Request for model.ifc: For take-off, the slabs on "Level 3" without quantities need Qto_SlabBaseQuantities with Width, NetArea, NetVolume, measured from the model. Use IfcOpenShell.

First a look at what the model holds.

```python
import ifcopenshell
import ifcopenshell.util.element
import ifcopenshell.util.unit

model = ifcopenshell.open("model.ifc")
print(model.schema)
for unit_type in ("LENGTHUNIT", "AREAUNIT", "VOLUMEUNIT"):
    print(unit_type, ifcopenshell.util.unit.calculate_unit_scale(model, unit_type))
storey = next(s for s in model.by_type("IfcBuildingStorey") if s.Name == "Level 3")
slabs = [e for e in ifcopenshell.util.element.get_decomposition(storey) if e.is_a("IfcSlab")]
for e in sorted(slabs, key=lambda e: e.id()):
    print(e.id(), e.is_a(), e.Name, list(ifcopenshell.util.element.get_psets(e, qtos_only=True)), sep=" | ")
```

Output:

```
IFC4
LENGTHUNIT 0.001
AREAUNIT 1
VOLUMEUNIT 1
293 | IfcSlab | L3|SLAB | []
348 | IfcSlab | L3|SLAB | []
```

```python
import ifcopenshell
import ifcopenshell.api.pset
import ifcopenshell.geom
import ifcopenshell.util.element
import ifcopenshell.util.shape
import ifcopenshell.util.unit

model = ifcopenshell.open("model.ifc")
unit_scale = ifcopenshell.util.unit.calculate_unit_scale(model)
area_scale = ifcopenshell.util.unit.calculate_unit_scale(model, "AREAUNIT")
volume_scale = ifcopenshell.util.unit.calculate_unit_scale(model, "VOLUMEUNIT")
settings = ifcopenshell.geom.settings()

storey = next(s for s in model.by_type("IfcBuildingStorey") if s.Name == "Level 3")
slabs = [e for e in ifcopenshell.util.element.get_decomposition(storey) if e.is_a("IfcSlab")]

for e in sorted(slabs, key=lambda e: e.id()):
    if ifcopenshell.util.element.get_psets(e, qtos_only=True, should_inherit=False):
        continue
    # Geometry comes back in metres, in the element's own axes.
    shape = ifcopenshell.geom.create_shape(settings, e)
    values = {
        "Width": ifcopenshell.util.shape.get_z(shape.geometry) / unit_scale,
        "NetArea": ifcopenshell.util.shape.get_footprint_area(shape.geometry) / area_scale,
        "NetVolume": ifcopenshell.util.shape.get_volume(shape.geometry) / volume_scale,
    }
    qto = ifcopenshell.api.pset.add_qto(model, product=e, name="Qto_SlabBaseQuantities")
    ifcopenshell.api.pset.edit_qto(model, qto=qto, properties=values)
    print(e.id(), {k: round(v, 3) for k, v in values.items()})

model.write("model_edited.ifc")
```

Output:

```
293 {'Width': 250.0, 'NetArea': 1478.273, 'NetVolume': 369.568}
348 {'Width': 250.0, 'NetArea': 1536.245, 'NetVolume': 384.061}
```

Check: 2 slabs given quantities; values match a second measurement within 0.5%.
